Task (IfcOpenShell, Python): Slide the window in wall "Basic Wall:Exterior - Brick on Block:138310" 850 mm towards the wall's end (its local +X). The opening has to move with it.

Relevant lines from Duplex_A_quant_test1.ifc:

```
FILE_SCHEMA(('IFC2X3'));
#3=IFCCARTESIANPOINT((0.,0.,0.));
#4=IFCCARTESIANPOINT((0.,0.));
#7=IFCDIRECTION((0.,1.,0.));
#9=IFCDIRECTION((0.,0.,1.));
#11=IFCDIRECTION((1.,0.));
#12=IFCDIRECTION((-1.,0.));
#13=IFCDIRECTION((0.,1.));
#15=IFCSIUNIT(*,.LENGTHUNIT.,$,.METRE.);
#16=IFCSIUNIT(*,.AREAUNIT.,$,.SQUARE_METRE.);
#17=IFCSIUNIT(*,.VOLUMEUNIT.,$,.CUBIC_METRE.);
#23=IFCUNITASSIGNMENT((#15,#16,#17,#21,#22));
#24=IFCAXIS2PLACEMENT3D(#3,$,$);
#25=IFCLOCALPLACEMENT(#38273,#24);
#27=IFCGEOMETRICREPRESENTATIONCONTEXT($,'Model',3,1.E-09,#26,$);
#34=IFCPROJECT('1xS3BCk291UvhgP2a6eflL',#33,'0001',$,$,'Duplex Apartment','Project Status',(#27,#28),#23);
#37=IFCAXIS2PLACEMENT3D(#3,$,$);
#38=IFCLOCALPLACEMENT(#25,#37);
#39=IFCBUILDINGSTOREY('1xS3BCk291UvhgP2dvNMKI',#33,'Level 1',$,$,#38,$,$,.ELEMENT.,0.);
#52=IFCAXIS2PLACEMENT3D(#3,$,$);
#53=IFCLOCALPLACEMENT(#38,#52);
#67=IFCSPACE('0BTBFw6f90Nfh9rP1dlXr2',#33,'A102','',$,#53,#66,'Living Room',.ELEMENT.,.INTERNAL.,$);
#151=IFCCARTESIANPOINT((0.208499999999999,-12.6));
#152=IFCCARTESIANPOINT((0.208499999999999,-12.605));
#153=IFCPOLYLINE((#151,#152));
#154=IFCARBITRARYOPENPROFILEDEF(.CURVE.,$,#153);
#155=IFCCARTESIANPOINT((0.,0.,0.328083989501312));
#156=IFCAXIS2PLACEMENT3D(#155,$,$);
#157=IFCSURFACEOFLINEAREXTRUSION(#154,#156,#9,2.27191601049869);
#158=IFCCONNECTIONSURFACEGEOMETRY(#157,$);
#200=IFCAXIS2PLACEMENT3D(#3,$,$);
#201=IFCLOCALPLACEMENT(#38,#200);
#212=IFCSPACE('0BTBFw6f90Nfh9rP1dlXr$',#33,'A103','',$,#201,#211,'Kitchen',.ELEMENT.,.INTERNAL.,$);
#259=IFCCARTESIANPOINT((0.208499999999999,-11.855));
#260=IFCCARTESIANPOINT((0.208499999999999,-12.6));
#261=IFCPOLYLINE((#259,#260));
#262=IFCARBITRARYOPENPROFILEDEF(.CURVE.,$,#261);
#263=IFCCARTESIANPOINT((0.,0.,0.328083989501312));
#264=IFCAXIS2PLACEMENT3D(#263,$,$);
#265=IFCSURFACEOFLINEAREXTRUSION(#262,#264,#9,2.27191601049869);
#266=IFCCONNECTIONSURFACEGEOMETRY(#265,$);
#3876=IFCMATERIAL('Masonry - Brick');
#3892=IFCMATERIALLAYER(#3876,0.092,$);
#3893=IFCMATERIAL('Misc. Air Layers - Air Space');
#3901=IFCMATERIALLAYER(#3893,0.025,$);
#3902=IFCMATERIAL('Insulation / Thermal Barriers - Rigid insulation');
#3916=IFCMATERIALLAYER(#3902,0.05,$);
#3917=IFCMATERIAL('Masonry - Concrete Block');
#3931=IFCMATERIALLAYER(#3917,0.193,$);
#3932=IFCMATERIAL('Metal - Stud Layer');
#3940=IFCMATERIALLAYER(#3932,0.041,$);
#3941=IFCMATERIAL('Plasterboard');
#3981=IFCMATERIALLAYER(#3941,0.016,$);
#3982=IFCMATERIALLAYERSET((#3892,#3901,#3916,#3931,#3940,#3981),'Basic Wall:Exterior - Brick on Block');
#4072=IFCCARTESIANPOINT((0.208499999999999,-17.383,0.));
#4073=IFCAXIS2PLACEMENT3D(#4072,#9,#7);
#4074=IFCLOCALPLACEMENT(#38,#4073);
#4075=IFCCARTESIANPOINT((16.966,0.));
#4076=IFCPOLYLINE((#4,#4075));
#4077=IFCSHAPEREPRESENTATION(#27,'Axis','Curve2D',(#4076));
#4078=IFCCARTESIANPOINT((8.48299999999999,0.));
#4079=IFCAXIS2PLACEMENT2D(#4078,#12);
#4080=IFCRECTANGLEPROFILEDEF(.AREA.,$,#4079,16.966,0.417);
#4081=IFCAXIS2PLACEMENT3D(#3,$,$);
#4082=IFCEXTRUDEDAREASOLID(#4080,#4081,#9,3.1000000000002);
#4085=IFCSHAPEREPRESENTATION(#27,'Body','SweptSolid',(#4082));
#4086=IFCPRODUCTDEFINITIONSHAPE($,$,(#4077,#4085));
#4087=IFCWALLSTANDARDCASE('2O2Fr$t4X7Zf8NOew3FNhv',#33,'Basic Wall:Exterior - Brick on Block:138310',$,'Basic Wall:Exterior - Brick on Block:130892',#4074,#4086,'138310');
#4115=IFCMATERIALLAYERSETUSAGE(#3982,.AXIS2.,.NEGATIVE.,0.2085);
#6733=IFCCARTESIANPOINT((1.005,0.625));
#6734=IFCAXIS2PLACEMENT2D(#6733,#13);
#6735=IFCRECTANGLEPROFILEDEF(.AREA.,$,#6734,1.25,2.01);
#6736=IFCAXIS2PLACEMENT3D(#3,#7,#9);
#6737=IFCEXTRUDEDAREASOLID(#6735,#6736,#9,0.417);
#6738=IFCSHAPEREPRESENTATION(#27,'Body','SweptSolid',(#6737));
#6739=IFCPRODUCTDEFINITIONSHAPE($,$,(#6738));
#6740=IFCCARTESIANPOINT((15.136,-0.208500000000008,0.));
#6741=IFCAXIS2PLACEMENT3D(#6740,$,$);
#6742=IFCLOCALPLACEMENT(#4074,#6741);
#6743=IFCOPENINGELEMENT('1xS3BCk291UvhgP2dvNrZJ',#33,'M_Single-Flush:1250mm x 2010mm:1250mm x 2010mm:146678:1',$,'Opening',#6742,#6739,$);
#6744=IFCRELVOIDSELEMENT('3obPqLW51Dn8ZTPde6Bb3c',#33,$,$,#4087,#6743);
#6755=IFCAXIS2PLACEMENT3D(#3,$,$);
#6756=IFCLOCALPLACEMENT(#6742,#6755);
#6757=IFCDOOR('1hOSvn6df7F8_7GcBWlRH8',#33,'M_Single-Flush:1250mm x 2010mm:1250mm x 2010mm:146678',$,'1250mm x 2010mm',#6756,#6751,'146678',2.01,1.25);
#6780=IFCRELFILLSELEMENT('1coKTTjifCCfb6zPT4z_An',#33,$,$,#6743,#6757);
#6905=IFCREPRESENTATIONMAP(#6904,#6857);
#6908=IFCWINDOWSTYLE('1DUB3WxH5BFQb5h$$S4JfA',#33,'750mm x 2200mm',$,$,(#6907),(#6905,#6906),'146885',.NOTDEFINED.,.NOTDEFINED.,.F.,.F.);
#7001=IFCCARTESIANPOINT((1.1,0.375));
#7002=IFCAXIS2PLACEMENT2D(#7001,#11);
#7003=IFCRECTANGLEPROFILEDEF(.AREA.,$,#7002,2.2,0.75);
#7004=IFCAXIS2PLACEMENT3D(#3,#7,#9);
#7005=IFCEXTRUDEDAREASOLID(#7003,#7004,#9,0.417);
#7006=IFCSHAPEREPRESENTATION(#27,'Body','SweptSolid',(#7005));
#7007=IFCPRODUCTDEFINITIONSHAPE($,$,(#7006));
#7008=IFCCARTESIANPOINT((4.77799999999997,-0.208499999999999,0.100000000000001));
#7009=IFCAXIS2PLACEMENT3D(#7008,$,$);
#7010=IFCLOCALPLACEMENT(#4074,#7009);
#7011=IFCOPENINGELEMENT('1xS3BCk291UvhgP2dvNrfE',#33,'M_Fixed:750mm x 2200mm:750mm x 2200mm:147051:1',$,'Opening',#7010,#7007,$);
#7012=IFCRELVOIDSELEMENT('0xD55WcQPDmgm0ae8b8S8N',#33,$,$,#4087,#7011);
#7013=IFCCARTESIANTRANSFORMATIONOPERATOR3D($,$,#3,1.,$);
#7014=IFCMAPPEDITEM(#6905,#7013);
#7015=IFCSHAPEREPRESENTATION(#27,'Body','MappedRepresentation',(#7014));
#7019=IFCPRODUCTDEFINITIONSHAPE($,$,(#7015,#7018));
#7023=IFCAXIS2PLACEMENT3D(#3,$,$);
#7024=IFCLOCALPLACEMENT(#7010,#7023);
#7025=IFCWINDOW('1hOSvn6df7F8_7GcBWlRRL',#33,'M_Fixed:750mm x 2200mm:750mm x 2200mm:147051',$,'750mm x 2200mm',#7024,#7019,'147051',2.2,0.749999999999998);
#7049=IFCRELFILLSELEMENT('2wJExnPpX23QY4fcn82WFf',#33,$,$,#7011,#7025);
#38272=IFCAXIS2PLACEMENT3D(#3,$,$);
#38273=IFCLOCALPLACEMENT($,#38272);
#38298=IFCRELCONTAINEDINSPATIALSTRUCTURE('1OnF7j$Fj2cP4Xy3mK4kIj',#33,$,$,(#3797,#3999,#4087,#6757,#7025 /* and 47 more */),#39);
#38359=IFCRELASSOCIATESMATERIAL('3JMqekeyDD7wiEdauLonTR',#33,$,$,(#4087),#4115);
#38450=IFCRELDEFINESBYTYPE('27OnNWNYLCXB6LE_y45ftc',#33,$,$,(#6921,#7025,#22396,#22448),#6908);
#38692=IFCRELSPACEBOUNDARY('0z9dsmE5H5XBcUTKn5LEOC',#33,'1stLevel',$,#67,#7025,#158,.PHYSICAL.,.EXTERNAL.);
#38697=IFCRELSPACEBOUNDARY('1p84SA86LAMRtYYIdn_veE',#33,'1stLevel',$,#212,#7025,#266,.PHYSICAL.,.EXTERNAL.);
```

```python
import numpy as np
import ifcopenshell
import ifcopenshell.api.geometry
import ifcopenshell.util.placement

model = ifcopenshell.open("Duplex_A_quant_test1.ifc")

window = model.by_guid("1hOSvn6df7F8_7GcBWlRRL")
opening = window.FillsVoids[0].RelatingOpeningElement
wall = opening.VoidsElements[0].RelatingBuildingElement

wall_matrix = ifcopenshell.util.placement.get_local_placement(wall.ObjectPlacement)
shift = wall_matrix[:3, 0] * 0.85
before = ifcopenshell.util.placement.get_local_placement(window.ObjectPlacement)[:3, 3].copy()

# The window is placed relative to its opening, so it follows when the opening moves.
matrix = ifcopenshell.util.placement.get_local_placement(opening.ObjectPlacement)
matrix[:3, 3] += shift
ifcopenshell.api.geometry.edit_object_placement(
    model, product=opening, matrix=matrix, is_si=False, should_transform_children=True
)

# Space boundary surfaces are stored in each space's coordinates; move them too.
for rel in window.ProvidesBoundaries:
    if not rel.ConnectionGeometry:
        continue
    surface = rel.ConnectionGeometry.SurfaceOnRelatingElement
    space_matrix = ifcopenshell.util.placement.get_local_placement(rel.RelatingSpace.ObjectPlacement)
    point = np.array(surface.Position.Location.Coordinates) + space_matrix[:3, :3].T @ shift
    surface.Position = model.createIfcAxis2Placement3D(
        model.createIfcCartesianPoint(point.tolist()), surface.Position.Axis, surface.Position.RefDirection
    )

after = ifcopenshell.util.placement.get_local_placement(window.ObjectPlacement)[:3, 3]
print("window moved by", (after - before).round(3) + 0.0)

model.write("Duplex_A_quant_test1_v2.ifc")
```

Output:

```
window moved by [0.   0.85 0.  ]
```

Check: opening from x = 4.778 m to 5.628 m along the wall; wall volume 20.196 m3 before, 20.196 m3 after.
